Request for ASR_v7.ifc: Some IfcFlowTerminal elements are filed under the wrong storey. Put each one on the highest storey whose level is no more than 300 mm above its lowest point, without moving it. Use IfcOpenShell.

First a look at what the model holds.

```python
import ifcopenshell
import ifcopenshell.util.element
import ifcopenshell.util.placement

model = ifcopenshell.open("ASR_v7.ifc")
print(model.schema)
for storey in model.by_type("IfcBuildingStorey"):
    level = ifcopenshell.util.placement.get_storey_elevation(storey)
    count = sum(e.is_a("IfcFlowTerminal") for e in ifcopenshell.util.element.get_contained(storey))
    print(storey.id(), storey.Name, round(level, 3), count, sep=" | ")
```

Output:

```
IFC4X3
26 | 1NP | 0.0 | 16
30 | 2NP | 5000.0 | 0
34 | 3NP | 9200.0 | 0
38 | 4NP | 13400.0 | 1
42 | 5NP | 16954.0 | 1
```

```python
import ifcopenshell
import ifcopenshell.api.spatial
import ifcopenshell.geom
import ifcopenshell.util.element
import ifcopenshell.util.placement
import ifcopenshell.util.shape
import ifcopenshell.util.unit

model = ifcopenshell.open("ASR_v7.ifc")
unit_scale = ifcopenshell.util.unit.calculate_unit_scale(model)
settings = ifcopenshell.geom.settings()

levels = sorted(
    ((ifcopenshell.util.placement.get_storey_elevation(s) * unit_scale, s) for s in model.by_type("IfcBuildingStorey")),
    key=lambda pair: pair[0],
)

for e in model.by_type("IfcFlowTerminal"):
    current = e.ContainedInStructure[0].RelatingStructure if e.ContainedInStructure else None
    if current is None or not current.is_a("IfcBuildingStorey"):
        continue
    shape = ifcopenshell.geom.create_shape(settings, e)
    bottom = ifcopenshell.util.shape.get_shape_bottom_elevation(shape, shape.geometry)
    below = [s for level, s in levels if level <= bottom + 0.3]
    storey = below[-1] if below else levels[0][1]
    if storey != current:
        # assign_container keeps the world position.
        ifcopenshell.api.spatial.assign_container(model, products=[e], relating_structure=storey)
        print(e.id(), current.Name, "->", storey.Name)

model.write("ASR_v7_v2.ifc")
```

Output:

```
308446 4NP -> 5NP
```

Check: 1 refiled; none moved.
